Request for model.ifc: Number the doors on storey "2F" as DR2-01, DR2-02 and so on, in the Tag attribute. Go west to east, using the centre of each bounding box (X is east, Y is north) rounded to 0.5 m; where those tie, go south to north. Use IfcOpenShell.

First a look at what the model holds.

```python
import ifcopenshell
import ifcopenshell.util.element
import ifcopenshell.util.placement

model = ifcopenshell.open("model.ifc")
print(model.schema)
storey = next(s for s in model.by_type("IfcBuildingStorey") if s.Name == "2F")
doors = [e for e in ifcopenshell.util.element.get_decomposition(storey) if e.is_a("IfcDoor")]
for e in sorted(doors, key=lambda e: e.id()):
    origin = ifcopenshell.util.placement.get_local_placement(e.ObjectPlacement)[:3, 3]
    print(e.id(), e.Tag, e.Name, origin.round(2) + 0.0, sep=" | ")
```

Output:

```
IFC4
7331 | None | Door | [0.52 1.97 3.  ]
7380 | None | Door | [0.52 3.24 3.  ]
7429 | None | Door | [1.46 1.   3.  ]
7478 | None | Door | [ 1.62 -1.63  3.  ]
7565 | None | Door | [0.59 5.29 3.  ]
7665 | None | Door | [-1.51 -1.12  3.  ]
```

```python
import ifcopenshell
import ifcopenshell.geom
import ifcopenshell.util.element
import ifcopenshell.util.shape

model = ifcopenshell.open("model.ifc")
settings = ifcopenshell.geom.settings()
settings.set("use-world-coords", True)


def centre(element):
    shape = ifcopenshell.geom.create_shape(settings, element)
    return ifcopenshell.util.shape.get_bbox_centroid(shape.geometry)


storey = next(s for s in model.by_type("IfcBuildingStorey") if s.Name == "2F")
doors = [e for e in ifcopenshell.util.element.get_decomposition(storey) if e.is_a("IfcDoor")]

# Insertion points can sit at a corner or the storey origin, so sort by the geometry (in metres).
centres = {e: centre(e) for e in doors}
doors.sort(key=lambda e: (round(centres[e][0] / 0.5), centres[e][1]))

for i, e in enumerate(doors, start=1):
    number = f"DR2-{i:02d}"
    e.Tag = number
    print(e.id(), number)

model.write("model_v2.ifc")
```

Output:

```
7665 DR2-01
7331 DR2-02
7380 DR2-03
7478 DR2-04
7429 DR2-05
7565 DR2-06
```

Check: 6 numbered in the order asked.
